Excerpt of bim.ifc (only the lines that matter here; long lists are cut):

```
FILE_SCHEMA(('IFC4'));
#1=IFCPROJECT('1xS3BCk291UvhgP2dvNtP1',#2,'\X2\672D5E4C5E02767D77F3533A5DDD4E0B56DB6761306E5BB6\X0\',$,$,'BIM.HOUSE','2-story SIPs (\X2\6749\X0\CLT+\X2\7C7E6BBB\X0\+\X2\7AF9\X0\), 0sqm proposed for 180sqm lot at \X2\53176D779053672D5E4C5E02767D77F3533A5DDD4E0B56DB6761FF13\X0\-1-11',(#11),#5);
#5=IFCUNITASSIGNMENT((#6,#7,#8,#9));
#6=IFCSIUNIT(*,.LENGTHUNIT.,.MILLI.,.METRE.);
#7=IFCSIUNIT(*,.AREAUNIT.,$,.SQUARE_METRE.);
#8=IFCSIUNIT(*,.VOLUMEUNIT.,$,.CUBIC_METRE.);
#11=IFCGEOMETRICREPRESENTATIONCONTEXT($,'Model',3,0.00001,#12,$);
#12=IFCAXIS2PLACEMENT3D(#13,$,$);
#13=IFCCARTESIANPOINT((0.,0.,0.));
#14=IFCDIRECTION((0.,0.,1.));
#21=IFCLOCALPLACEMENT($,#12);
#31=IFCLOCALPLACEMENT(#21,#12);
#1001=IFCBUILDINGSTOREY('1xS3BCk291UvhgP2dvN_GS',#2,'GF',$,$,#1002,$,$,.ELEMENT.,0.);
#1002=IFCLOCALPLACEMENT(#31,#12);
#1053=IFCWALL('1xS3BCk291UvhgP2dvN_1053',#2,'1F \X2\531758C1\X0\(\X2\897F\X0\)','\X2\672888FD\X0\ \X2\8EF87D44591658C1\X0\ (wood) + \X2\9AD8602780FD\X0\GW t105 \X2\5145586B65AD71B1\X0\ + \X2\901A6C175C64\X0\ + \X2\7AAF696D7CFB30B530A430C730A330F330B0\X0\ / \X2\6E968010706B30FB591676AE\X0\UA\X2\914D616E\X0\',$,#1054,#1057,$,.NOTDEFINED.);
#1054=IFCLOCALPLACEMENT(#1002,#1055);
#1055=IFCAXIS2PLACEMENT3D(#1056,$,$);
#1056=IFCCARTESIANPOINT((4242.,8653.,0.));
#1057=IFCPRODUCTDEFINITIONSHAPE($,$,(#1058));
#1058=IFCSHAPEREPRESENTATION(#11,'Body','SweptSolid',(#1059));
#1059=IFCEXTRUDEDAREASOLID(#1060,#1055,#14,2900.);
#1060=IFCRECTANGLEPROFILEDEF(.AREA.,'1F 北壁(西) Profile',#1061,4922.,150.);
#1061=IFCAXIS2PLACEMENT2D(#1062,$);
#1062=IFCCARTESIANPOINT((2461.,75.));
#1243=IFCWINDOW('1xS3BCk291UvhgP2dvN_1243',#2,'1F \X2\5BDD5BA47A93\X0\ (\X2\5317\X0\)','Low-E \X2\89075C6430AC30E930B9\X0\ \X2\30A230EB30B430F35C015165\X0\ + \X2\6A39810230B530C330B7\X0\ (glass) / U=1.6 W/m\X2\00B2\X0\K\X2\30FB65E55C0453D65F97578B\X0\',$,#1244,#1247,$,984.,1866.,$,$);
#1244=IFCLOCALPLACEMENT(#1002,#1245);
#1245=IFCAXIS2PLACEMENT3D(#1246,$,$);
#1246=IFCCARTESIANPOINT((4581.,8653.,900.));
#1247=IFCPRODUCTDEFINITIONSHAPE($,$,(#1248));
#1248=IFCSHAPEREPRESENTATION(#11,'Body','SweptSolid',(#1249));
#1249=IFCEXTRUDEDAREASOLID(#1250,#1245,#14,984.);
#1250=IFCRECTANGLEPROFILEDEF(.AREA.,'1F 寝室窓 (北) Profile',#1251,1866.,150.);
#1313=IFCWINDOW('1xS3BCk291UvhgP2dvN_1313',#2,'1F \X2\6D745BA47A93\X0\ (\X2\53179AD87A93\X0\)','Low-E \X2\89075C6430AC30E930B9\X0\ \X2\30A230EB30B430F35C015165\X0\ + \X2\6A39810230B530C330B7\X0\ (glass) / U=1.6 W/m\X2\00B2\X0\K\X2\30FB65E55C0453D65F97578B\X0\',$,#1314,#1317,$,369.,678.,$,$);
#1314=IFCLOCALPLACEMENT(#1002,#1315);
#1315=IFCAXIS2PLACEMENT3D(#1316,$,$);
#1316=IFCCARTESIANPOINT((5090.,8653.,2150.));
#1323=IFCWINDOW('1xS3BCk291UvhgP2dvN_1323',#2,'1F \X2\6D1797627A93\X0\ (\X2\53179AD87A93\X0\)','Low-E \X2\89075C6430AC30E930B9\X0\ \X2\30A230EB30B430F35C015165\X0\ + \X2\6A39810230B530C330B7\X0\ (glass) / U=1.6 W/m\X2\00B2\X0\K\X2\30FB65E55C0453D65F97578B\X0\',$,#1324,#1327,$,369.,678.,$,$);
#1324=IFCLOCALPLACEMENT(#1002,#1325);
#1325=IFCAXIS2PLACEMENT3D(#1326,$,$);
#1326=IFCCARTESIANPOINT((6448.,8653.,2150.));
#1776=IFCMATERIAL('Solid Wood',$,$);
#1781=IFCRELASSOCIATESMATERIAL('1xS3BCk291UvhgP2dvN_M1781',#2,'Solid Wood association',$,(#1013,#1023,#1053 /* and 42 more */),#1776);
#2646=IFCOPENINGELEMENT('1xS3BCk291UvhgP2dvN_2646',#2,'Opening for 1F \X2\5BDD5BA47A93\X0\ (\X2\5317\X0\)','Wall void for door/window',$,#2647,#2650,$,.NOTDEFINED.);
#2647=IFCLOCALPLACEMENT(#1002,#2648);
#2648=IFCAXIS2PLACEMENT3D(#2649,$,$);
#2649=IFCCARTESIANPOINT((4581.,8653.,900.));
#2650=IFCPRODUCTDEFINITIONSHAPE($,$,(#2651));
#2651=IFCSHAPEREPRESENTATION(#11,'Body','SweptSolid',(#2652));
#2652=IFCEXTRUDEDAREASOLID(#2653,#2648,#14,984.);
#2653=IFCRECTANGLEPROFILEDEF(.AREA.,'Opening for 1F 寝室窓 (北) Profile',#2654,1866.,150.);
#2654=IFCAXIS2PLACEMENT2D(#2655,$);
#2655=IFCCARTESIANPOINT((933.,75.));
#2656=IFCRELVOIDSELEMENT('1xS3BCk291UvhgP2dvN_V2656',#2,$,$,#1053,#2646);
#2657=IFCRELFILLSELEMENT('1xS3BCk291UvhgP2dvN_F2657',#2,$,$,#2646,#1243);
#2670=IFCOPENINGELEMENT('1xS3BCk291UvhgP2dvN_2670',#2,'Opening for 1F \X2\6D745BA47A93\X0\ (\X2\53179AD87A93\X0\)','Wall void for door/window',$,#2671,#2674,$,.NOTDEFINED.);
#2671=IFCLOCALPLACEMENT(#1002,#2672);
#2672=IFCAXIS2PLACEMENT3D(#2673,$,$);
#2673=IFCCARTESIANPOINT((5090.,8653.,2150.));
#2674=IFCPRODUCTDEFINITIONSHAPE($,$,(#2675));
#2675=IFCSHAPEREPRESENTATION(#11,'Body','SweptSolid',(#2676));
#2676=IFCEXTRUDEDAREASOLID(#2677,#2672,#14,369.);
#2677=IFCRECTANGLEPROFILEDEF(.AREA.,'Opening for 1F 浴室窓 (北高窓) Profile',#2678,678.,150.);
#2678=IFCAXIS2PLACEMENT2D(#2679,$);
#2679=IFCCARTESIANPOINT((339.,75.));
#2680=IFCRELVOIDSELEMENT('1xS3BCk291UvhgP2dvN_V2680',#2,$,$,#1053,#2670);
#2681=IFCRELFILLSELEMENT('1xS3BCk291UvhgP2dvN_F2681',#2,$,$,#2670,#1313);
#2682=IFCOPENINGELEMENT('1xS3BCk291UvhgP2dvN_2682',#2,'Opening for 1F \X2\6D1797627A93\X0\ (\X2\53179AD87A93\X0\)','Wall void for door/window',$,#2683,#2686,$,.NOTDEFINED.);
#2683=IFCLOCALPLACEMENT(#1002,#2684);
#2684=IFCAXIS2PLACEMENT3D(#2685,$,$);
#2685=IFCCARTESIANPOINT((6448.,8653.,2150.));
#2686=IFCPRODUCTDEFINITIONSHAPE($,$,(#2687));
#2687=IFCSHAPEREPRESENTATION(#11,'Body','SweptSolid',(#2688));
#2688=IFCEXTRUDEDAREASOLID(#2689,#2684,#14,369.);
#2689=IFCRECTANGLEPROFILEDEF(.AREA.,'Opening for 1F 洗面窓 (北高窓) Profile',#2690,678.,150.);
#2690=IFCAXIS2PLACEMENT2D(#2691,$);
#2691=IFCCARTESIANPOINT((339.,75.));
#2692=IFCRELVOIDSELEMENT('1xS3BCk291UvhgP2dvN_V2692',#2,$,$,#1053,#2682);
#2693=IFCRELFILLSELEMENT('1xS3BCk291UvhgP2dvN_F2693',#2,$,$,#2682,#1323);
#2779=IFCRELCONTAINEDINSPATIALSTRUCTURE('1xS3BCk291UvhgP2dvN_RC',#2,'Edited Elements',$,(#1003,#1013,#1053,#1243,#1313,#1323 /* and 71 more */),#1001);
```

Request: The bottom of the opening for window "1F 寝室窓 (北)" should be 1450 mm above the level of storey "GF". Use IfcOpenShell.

```python
import numpy as np
import ifcopenshell
import ifcopenshell.api.geometry
import ifcopenshell.geom
import ifcopenshell.util.element
import ifcopenshell.util.placement
import ifcopenshell.util.shape
import ifcopenshell.util.unit

model = ifcopenshell.open("bim.ifc")
unit_scale = ifcopenshell.util.unit.calculate_unit_scale(model)

window = model.by_id(1243)
opening = window.FillsVoids[0].RelatingOpeningElement
storey = ifcopenshell.util.element.get_container(window, ifc_class="IfcBuildingStorey")
level = ifcopenshell.util.placement.get_local_placement(storey.ObjectPlacement)[2, 3]

# The opening's origin need not be at the sill, so measure its lowest point.
shape = ifcopenshell.geom.create_shape(ifcopenshell.geom.settings(), opening)
bottom = ifcopenshell.util.shape.get_shape_bottom_elevation(shape, shape.geometry) / unit_scale
dz = level + 1.45 / unit_scale - bottom

shift = np.array([0.0, 0.0, dz])
# The window is not placed relative to its opening, so move both.
for product in (opening, window):
    matrix = ifcopenshell.util.placement.get_local_placement(product.ObjectPlacement)
    matrix[:3, 3] += shift
    ifcopenshell.api.geometry.edit_object_placement(model, product=product, matrix=matrix, is_si=False)

print(f"moved by {dz * unit_scale:+.3f} m")

model.write("bim_updated.ifc")
```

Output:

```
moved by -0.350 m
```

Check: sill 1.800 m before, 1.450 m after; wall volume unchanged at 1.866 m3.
